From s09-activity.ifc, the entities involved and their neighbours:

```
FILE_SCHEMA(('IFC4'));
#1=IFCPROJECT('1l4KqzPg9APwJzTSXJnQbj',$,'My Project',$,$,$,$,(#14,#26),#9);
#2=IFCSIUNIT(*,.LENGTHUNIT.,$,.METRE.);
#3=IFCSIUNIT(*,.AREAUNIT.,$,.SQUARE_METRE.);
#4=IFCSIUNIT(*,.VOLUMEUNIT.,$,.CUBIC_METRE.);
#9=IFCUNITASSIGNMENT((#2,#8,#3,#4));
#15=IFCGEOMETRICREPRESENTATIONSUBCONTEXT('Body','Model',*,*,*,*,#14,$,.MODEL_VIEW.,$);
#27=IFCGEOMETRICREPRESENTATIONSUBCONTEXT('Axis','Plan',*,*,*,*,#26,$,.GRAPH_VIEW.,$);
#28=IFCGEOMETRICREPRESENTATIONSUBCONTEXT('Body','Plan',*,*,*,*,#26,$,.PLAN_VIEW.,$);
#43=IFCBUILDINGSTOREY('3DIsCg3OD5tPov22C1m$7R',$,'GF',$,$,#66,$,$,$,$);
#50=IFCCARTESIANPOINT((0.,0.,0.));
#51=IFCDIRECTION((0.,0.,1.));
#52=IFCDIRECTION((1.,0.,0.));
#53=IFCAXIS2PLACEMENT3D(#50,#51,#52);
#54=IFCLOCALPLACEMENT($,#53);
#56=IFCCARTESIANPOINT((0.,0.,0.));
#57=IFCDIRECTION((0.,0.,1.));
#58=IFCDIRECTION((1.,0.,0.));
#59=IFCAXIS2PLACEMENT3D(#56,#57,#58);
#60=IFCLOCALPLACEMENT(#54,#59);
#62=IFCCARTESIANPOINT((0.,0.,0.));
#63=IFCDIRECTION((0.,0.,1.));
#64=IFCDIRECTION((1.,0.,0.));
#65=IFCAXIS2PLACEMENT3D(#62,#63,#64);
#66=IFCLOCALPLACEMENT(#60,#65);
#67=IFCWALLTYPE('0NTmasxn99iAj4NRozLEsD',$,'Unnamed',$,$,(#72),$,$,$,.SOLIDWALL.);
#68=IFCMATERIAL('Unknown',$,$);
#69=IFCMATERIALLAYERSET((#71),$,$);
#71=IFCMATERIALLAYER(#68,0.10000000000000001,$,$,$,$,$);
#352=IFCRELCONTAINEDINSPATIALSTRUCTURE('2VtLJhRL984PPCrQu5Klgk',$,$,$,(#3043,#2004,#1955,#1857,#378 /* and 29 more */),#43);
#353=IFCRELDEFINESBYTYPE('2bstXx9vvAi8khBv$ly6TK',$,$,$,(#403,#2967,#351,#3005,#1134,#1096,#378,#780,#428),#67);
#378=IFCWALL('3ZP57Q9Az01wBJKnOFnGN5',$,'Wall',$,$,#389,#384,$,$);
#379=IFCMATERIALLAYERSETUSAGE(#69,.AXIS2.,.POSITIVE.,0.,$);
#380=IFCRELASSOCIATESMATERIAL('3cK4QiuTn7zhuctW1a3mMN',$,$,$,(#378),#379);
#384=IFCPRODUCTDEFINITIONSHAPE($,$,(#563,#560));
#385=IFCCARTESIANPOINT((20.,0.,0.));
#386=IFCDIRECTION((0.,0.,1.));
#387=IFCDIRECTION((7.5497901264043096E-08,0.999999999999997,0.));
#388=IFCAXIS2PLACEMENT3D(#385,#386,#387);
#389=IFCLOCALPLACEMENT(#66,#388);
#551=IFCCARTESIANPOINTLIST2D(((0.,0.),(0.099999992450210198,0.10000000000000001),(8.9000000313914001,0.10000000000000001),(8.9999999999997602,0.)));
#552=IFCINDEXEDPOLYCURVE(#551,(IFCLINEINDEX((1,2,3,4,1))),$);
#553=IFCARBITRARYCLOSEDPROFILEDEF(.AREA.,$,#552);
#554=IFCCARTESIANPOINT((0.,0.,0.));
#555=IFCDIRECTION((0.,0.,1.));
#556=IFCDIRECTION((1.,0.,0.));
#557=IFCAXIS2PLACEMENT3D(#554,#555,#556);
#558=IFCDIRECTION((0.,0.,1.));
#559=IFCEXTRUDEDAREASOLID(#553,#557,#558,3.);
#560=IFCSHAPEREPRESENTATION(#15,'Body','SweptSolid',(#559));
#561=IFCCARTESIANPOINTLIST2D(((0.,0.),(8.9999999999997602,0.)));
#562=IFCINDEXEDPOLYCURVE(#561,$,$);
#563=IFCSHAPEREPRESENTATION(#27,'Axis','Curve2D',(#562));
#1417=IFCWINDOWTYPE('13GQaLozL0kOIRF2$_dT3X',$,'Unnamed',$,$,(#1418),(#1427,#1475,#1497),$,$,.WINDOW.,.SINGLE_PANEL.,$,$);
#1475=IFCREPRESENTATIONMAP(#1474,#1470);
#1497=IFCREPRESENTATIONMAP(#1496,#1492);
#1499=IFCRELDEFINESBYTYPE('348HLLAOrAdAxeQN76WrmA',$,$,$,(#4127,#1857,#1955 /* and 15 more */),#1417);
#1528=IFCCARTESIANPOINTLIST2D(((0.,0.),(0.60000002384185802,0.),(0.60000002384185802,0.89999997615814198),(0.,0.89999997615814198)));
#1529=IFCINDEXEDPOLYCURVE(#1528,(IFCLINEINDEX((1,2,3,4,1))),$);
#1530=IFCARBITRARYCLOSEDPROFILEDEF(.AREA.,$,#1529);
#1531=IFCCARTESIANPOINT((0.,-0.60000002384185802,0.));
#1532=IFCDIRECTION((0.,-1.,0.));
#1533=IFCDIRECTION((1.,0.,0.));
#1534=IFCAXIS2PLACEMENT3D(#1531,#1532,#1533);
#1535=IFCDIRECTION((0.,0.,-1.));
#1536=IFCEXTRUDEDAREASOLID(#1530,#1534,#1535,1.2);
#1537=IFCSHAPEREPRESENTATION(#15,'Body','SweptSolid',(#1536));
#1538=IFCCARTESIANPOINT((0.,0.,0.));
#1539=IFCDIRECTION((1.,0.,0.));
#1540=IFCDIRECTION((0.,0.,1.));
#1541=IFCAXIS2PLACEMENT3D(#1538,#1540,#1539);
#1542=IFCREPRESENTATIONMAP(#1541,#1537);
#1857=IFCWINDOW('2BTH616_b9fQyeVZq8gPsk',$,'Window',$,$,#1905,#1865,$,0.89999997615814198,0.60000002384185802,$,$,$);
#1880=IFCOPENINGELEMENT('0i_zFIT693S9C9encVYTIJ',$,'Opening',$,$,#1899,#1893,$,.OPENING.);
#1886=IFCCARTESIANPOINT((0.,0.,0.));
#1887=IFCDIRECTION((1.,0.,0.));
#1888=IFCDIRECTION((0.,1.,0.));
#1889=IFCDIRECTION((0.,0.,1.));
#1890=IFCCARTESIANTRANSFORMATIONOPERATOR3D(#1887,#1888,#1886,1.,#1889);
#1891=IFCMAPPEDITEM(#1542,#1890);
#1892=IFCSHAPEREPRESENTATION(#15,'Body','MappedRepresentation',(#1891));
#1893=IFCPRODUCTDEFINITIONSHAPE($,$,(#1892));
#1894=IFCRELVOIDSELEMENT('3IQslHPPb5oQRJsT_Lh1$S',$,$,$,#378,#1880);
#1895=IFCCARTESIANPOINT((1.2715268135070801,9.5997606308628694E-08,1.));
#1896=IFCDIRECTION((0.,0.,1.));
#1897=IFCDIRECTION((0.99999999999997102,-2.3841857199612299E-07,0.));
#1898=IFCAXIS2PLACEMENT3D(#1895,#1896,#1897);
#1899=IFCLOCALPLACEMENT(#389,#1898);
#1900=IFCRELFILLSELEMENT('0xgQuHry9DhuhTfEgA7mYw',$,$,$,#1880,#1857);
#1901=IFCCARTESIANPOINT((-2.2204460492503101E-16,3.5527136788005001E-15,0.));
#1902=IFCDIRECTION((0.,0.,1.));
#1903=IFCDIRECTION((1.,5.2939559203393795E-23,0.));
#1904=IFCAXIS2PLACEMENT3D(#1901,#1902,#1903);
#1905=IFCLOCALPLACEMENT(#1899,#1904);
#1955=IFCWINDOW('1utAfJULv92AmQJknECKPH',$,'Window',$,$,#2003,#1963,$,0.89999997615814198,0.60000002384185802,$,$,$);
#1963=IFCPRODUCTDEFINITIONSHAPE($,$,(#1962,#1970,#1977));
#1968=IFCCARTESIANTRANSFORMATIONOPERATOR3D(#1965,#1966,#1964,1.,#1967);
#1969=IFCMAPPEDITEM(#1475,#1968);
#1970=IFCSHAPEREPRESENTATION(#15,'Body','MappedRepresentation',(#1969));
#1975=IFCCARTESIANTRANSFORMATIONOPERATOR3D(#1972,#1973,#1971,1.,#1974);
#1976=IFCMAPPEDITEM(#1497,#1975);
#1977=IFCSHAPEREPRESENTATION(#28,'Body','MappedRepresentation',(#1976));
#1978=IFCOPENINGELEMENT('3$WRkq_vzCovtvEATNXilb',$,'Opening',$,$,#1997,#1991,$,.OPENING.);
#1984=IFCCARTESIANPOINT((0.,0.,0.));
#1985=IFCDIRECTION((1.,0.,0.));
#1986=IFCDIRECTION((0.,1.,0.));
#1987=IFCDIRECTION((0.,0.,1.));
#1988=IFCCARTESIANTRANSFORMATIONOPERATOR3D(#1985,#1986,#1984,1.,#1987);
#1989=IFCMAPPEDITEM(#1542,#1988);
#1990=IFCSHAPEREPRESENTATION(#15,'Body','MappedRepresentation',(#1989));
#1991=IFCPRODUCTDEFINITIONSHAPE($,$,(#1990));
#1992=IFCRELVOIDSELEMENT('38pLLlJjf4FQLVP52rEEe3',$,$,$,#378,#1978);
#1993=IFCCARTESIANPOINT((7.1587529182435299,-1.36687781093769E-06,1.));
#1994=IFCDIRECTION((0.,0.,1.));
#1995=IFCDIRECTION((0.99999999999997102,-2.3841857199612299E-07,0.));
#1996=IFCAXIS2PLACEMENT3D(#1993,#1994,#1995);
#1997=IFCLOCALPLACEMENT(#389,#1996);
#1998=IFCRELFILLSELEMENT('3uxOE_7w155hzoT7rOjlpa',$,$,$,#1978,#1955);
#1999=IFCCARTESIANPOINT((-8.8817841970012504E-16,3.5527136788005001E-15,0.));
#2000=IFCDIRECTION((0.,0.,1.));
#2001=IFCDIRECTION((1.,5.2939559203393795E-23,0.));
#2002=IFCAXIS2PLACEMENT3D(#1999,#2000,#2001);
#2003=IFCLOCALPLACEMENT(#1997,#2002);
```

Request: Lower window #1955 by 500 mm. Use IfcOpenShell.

```python
import numpy as np
import ifcopenshell
import ifcopenshell.api.geometry
import ifcopenshell.util.placement
import ifcopenshell.util.unit

model = ifcopenshell.open("s09-activity.ifc")
unit_scale = ifcopenshell.util.unit.calculate_unit_scale(model)

window = model.by_id(1955)
opening = window.FillsVoids[0].RelatingOpeningElement
dz = -0.5

shift = np.array([0.0, 0.0, dz])
# The window is placed relative to its opening, so it follows when the opening moves.
matrix = ifcopenshell.util.placement.get_local_placement(opening.ObjectPlacement)
matrix[:3, 3] += shift
ifcopenshell.api.geometry.edit_object_placement(
    model, product=opening, matrix=matrix, is_si=False, should_transform_children=True
)

print(f"moved by {dz * unit_scale:+.3f} m")

model.write("s09-activity_edited.ifc")
```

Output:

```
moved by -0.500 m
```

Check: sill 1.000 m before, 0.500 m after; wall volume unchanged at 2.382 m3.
